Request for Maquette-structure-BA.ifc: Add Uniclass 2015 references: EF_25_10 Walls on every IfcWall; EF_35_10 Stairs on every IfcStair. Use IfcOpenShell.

First a look at what the model holds.

```python
import ifcopenshell

model = ifcopenshell.open("Maquette-structure-BA.ifc")
print(model.schema)
print("classifications:", [c.Name for c in model.by_type("IfcClassification")])
for ifc_class in ("IfcDoor", "IfcRoof", "IfcStair", "IfcWall", "IfcWindow"):
    print(ifc_class, len(model.by_type(ifc_class)))
```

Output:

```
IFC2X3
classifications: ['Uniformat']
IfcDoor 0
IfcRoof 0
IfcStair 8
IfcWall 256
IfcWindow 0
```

```python
import ifcopenshell
import ifcopenshell.api.classification

model = ifcopenshell.open("Maquette-structure-BA.ifc")

# IFC2X3 requires Source and Edition and has no link from the project to the system.
system = model.create_entity("IfcClassification", Source="NBS", Edition="2015", Name="Uniclass 2015")

codes = {
    "IfcWall": ("EF_25_10", "Walls"),
    "IfcStair": ("EF_35_10", "Stairs"),
}
for ifc_class, (code, name) in codes.items():
    products = model.by_type(ifc_class)
    ifcopenshell.api.classification.add_reference(
        model, products=products, classification=system, identification=code, name=name
    )
    print(code, len(products))

model.write("Maquette-structure-BA_rev.ifc")
```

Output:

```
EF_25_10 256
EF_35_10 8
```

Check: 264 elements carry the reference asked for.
